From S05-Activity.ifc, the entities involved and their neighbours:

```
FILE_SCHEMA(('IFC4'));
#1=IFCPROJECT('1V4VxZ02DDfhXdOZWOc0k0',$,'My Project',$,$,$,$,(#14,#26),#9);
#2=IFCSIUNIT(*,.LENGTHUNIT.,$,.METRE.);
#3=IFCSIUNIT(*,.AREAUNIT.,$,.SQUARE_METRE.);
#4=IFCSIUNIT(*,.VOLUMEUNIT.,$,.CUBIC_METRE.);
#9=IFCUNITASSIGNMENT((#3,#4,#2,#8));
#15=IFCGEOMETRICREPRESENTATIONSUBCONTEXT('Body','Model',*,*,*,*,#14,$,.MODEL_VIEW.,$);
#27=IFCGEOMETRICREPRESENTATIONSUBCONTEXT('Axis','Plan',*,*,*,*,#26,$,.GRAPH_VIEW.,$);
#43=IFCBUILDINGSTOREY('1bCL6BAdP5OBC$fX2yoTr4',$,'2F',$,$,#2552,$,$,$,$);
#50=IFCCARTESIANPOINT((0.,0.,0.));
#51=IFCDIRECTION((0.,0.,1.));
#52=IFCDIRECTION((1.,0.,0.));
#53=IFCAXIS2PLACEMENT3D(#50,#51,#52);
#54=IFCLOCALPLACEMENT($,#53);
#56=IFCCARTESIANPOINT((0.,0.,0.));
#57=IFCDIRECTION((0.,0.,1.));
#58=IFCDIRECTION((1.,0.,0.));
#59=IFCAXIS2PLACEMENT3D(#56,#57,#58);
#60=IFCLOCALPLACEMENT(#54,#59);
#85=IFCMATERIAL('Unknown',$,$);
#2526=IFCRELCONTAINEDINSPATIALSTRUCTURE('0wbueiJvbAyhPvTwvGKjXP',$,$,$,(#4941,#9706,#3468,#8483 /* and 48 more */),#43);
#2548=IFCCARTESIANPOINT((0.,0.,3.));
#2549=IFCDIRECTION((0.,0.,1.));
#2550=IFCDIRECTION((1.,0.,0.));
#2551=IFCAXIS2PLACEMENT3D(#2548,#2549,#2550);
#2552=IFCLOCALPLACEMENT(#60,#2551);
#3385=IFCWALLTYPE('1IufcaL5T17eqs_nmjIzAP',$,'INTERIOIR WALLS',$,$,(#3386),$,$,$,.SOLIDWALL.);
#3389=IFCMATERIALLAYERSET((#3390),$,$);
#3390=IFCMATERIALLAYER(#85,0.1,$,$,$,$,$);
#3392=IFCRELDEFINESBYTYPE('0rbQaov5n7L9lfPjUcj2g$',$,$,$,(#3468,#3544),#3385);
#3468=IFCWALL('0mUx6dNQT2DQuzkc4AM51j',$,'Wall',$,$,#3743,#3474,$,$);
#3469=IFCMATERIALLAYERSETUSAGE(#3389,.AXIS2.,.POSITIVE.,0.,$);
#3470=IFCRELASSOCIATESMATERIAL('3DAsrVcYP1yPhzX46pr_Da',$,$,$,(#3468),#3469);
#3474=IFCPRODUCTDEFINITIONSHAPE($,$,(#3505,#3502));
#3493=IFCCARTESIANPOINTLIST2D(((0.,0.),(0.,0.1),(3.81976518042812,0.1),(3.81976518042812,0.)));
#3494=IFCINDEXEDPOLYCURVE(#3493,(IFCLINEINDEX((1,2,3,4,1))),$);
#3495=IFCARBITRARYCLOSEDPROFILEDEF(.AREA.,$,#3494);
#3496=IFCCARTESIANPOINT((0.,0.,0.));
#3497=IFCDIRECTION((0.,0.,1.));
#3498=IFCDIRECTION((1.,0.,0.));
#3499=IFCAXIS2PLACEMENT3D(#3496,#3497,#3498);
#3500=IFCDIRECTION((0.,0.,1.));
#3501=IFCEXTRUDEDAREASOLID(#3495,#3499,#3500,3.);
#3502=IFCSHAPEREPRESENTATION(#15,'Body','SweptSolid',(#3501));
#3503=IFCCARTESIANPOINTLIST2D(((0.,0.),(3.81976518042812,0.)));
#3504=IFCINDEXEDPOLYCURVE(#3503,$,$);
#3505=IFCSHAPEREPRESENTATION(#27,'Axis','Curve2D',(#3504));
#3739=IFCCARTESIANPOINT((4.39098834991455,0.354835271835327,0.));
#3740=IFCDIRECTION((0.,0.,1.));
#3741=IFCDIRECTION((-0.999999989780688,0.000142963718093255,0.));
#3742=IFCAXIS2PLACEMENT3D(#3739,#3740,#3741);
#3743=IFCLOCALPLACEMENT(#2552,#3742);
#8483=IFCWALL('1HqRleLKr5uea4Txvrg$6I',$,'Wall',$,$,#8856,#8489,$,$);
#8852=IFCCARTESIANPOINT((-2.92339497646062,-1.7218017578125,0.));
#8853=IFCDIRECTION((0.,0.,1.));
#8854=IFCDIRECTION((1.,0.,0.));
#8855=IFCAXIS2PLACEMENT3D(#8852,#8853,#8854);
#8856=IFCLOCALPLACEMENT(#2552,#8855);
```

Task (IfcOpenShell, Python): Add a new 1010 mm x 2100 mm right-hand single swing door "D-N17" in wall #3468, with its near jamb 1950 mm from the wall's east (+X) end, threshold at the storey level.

```python
import numpy as np
import ifcopenshell
import ifcopenshell.api.feature
import ifcopenshell.api.geometry
import ifcopenshell.api.root
import ifcopenshell.api.spatial
import ifcopenshell.geom
import ifcopenshell.util.element
import ifcopenshell.util.placement
import ifcopenshell.util.representation
import ifcopenshell.util.shape
import ifcopenshell.util.unit

model = ifcopenshell.open("S05-Activity.ifc")
unit_scale = ifcopenshell.util.unit.calculate_unit_scale(model)
settings = ifcopenshell.geom.settings()


def volume(element):
    """Net volume in cubic metres, openings subtracted."""
    shape = ifcopenshell.geom.create_shape(settings, element)
    return ifcopenshell.util.shape.get_volume(shape.geometry)


wall = model.by_id(3468)
storey = ifcopenshell.util.element.get_container(wall, ifc_class="IfcBuildingStorey")
context = ifcopenshell.util.representation.get_context(model, "Model", "Body", "MODEL_VIEW")
before = volume(wall)

width, height, from_end, sill = 1.01, 2.1, 1.95, 0.0  # metres

# The wall runs along its own X axis, and the end named is its -X end.
wall_shape = ifcopenshell.geom.create_shape(settings, wall)
x, y, z = ifcopenshell.util.shape.get_vertices(wall_shape.geometry).T
start = x.min() + from_end
face, thickness = float(y.min()), float(y.max() - y.min())
wall_matrix = ifcopenshell.util.placement.get_local_placement(wall.ObjectPlacement)
level = ifcopenshell.util.placement.get_local_placement(storey.ObjectPlacement)[2, 3]


def in_wall(x, y):
    """Placement at x, y metres in the wall's axes, at sill height."""
    matrix = wall_matrix.copy()
    matrix[:, 3] = wall_matrix @ np.array([x / unit_scale, y / unit_scale, 0.0, 1.0])
    matrix[2, 3] = level + sill / unit_scale
    return matrix


# Opening: a box that overshoots both wall faces by 50 mm.
opening = ifcopenshell.api.root.create_entity(model, ifc_class="IfcOpeningElement", predefined_type="OPENING")
box = ifcopenshell.api.geometry.add_wall_representation(
    model, context=context, length=width, height=height, thickness=thickness + 0.1
)
ifcopenshell.api.geometry.assign_representation(model, product=opening, representation=box)
ifcopenshell.api.geometry.edit_object_placement(model, product=opening, matrix=in_wall(start, face - 0.05), is_si=False)
ifcopenshell.api.feature.add_feature(model, feature=opening, element=wall)

door = ifcopenshell.api.root.create_entity(model, ifc_class="IfcDoor", name="D-N17", predefined_type="DOOR")
door.OverallWidth, door.OverallHeight = width / unit_scale, height / unit_scale
door.OperationType = "SINGLE_SWING_RIGHT"
body = ifcopenshell.api.geometry.add_door_representation(
    model,
    context=context,
    overall_width=door.OverallWidth,
    overall_height=door.OverallHeight,
    operation_type="SINGLE_SWING_RIGHT",
    lining_properties={"LiningDepth": thickness / unit_scale, "ThresholdDepth": thickness / unit_scale},
)
ifcopenshell.api.geometry.assign_representation(model, product=door, representation=body)
ifcopenshell.api.spatial.assign_container(model, products=[door], relating_structure=storey)
ifcopenshell.api.feature.add_filling(model, opening=opening, element=door)

# The lining spans the wall, so the door starts at the wall face.
ifcopenshell.api.geometry.edit_object_placement(model, product=door, matrix=in_wall(start, face), is_si=False)

after = volume(wall)

print(f"wall volume {before:.3f} -> {after:.3f} m3")

model.write("S05-Activity-out.ifc")
```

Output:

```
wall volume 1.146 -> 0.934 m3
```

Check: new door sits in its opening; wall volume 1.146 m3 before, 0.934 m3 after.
